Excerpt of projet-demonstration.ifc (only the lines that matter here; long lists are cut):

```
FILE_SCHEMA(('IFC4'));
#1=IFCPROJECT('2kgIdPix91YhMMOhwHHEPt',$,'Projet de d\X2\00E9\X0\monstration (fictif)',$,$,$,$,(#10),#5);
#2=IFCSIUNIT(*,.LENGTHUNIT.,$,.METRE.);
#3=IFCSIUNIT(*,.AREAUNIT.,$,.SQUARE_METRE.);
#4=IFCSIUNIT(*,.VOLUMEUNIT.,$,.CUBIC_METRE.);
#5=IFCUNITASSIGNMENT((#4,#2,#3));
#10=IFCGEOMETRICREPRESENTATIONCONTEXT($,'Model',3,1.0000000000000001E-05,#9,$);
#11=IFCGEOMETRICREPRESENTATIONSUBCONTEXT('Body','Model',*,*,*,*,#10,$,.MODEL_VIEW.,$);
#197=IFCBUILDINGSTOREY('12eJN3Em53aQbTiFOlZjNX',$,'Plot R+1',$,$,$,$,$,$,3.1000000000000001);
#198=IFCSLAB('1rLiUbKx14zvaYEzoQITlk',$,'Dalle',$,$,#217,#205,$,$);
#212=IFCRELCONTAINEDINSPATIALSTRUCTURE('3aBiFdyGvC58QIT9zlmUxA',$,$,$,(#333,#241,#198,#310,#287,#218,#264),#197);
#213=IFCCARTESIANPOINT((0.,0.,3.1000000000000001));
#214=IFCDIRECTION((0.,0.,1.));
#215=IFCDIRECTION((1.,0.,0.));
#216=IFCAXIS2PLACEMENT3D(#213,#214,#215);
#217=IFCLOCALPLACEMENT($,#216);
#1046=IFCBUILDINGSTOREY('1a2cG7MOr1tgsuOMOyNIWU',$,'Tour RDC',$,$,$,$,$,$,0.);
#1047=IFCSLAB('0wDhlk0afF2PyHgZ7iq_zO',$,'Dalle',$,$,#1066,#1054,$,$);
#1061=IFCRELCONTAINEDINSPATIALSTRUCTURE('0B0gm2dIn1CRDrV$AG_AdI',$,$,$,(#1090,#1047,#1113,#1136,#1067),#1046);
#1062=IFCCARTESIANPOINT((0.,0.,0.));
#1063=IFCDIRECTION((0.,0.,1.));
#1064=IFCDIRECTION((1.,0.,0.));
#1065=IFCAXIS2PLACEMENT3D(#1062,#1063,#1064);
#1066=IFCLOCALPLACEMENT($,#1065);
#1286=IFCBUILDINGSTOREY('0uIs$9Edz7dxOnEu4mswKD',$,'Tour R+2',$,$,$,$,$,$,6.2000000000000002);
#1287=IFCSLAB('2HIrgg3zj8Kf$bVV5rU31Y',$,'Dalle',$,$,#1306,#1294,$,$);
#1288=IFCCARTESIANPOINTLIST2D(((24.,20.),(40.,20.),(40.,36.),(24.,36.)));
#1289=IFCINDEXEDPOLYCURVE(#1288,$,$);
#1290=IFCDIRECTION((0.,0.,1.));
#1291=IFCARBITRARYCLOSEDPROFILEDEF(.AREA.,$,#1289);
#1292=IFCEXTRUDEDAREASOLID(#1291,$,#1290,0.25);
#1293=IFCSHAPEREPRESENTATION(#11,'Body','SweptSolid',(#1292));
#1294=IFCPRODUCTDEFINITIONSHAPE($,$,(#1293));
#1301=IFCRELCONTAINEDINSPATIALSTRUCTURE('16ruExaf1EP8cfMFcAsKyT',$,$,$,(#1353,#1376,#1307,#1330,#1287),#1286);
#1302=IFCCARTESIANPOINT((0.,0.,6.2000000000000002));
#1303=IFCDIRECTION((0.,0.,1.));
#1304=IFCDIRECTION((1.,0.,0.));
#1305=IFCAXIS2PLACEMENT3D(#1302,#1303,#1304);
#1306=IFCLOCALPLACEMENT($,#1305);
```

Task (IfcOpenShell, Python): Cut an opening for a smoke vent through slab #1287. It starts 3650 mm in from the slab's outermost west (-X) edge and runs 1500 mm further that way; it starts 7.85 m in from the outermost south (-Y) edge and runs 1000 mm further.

```python
import numpy as np
import ifcopenshell
import ifcopenshell.api.feature
import ifcopenshell.api.geometry
import ifcopenshell.api.root
import ifcopenshell.geom
import ifcopenshell.util.placement
import ifcopenshell.util.representation
import ifcopenshell.util.shape
import ifcopenshell.util.unit

model = ifcopenshell.open("projet-demonstration.ifc")
unit_scale = ifcopenshell.util.unit.calculate_unit_scale(model)
settings = ifcopenshell.geom.settings()


def volume(element):
    """Net volume in cubic metres, openings subtracted."""
    shape = ifcopenshell.geom.create_shape(settings, element)
    return ifcopenshell.util.shape.get_volume(shape.geometry)


slab = model.by_guid("2HIrgg3zj8Kf$bVV5rU31Y")
before = volume(slab)

# Extent in the slab's own axes, in metres. The edges named are its -X and -Y sides.
slab_shape = ifcopenshell.geom.create_shape(settings, slab)
vertices = ifcopenshell.util.shape.get_vertices(slab_shape.geometry)
x_min, y_min, bottom = vertices.min(axis=0)
top = vertices[:, 2].max()

opening = ifcopenshell.api.root.create_entity(model, ifc_class="IfcOpeningElement", name="Smoke vent opening", predefined_type="OPENING")
context = ifcopenshell.util.representation.get_context(model, "Model", "Body", "MODEL_VIEW")
width, depth = 1.5, 1
outline = [(0.0, 0.0), (width, 0.0), (width, depth), (0.0, depth), (0.0, 0.0)]
# Overshoot both faces by 50 mm so the cut is clean.
shape = ifcopenshell.api.geometry.add_slab_representation(
    model, context=context, depth=top - bottom + 0.1, polyline=outline
)
ifcopenshell.api.geometry.assign_representation(model, product=opening, representation=shape)

matrix = ifcopenshell.util.placement.get_local_placement(slab.ObjectPlacement)
matrix[:, 3] = matrix @ np.append(np.array([x_min + 3.65, y_min + 7.85, bottom - 0.05]) / unit_scale, 1.0)
ifcopenshell.api.geometry.edit_object_placement(model, product=opening, matrix=matrix, is_si=False)
ifcopenshell.api.feature.add_feature(model, feature=opening, element=slab)

after = volume(slab)

print(f"slab volume {before:.3f} -> {after:.3f} m3")

model.write("projet-demonstration_edited.ifc")
```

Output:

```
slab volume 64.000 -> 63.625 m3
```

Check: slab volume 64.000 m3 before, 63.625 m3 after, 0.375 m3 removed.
